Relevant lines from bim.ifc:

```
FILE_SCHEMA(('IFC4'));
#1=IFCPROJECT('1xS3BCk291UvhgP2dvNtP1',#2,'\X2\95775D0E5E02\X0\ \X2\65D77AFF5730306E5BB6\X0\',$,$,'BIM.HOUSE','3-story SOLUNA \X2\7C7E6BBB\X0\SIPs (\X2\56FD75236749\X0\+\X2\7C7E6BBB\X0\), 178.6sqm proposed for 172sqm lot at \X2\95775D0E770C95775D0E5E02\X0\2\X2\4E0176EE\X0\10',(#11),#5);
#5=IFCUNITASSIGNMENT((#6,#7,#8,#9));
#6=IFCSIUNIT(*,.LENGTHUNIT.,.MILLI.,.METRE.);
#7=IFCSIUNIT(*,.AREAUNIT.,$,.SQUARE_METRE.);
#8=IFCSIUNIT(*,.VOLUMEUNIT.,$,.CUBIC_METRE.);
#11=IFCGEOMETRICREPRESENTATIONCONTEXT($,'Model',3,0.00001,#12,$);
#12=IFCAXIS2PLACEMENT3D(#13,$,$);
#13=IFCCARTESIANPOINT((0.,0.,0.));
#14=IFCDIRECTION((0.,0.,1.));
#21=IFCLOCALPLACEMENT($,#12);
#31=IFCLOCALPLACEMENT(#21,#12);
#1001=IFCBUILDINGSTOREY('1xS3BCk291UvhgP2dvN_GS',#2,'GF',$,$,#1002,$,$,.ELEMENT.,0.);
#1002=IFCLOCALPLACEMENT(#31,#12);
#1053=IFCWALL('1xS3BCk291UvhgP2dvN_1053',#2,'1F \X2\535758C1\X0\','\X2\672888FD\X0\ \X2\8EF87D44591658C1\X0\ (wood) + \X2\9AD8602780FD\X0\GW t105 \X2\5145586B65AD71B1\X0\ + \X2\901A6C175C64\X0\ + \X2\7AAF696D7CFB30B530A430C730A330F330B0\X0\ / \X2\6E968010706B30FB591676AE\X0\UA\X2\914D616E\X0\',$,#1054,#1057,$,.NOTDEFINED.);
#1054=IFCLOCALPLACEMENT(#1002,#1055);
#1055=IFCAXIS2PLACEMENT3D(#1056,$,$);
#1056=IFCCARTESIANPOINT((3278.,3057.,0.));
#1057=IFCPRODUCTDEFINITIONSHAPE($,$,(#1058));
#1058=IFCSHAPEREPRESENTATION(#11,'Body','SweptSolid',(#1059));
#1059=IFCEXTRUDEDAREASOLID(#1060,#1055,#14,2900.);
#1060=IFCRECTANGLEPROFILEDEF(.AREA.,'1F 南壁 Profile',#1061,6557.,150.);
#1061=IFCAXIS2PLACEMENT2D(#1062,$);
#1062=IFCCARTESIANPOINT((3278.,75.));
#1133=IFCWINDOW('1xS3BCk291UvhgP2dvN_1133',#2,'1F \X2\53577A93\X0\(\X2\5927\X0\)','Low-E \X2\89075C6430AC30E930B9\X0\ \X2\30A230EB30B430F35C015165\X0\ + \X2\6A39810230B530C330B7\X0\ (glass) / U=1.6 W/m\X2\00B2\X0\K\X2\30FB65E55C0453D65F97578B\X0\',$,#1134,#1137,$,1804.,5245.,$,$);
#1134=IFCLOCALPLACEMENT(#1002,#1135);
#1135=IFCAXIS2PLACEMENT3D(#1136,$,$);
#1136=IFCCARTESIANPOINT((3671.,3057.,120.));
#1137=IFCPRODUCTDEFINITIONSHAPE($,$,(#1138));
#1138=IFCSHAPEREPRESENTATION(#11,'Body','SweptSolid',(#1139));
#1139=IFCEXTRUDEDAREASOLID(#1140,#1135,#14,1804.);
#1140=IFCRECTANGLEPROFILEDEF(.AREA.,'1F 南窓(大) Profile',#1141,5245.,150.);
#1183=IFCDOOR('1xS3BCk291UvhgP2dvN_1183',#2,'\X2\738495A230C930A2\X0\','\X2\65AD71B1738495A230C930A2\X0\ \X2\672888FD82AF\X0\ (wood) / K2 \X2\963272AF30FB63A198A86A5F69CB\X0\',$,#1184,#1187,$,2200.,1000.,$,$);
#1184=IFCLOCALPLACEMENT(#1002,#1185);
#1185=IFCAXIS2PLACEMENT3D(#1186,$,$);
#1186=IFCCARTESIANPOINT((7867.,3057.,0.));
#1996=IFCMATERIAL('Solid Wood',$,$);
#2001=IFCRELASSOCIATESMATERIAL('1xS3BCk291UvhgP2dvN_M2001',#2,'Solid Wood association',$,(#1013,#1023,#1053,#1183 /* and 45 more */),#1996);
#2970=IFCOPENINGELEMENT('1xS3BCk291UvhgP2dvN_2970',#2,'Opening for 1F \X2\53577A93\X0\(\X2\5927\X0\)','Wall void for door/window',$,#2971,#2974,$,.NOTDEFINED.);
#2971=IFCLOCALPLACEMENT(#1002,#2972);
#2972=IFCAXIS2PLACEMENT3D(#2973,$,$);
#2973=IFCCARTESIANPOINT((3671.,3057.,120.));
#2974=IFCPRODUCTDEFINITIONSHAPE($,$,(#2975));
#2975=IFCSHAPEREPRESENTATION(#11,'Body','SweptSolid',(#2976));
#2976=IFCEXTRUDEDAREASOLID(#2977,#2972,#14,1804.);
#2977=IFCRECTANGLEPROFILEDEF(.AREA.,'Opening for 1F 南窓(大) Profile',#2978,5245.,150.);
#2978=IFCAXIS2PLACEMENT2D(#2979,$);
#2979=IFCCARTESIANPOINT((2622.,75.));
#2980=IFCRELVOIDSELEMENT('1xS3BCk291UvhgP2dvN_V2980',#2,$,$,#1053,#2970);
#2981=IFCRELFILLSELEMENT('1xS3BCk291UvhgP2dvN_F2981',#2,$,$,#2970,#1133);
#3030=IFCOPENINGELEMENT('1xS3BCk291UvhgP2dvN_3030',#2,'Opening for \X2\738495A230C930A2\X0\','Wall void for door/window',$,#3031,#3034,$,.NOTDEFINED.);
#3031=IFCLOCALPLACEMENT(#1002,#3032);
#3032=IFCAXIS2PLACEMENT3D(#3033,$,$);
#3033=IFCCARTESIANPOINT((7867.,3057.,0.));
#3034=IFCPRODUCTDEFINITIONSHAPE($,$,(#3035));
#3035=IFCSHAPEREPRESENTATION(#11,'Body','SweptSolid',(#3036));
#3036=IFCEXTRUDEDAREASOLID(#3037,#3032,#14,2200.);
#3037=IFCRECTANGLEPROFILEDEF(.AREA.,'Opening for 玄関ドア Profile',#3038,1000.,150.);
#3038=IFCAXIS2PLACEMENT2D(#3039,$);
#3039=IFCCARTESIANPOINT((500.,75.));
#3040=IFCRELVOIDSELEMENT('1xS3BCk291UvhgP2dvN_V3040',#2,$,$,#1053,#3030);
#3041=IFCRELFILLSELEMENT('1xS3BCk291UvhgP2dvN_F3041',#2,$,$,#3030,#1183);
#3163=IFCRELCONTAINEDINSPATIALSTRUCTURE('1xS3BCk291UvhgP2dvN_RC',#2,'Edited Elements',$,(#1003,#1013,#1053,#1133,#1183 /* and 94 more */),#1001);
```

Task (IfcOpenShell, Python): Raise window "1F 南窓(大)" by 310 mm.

```python
import numpy as np
import ifcopenshell
import ifcopenshell.api.geometry
import ifcopenshell.util.placement
import ifcopenshell.util.unit

model = ifcopenshell.open("bim.ifc")
unit_scale = ifcopenshell.util.unit.calculate_unit_scale(model)

window = model.by_id(1133)
opening = window.FillsVoids[0].RelatingOpeningElement
dz = 0.31 / unit_scale

shift = np.array([0.0, 0.0, dz])
# The window is not placed relative to its opening, so move both.
for product in (opening, window):
    matrix = ifcopenshell.util.placement.get_local_placement(product.ObjectPlacement)
    matrix[:3, 3] += shift
    ifcopenshell.api.geometry.edit_object_placement(model, product=product, matrix=matrix, is_si=False)

print(f"moved by {dz * unit_scale:+.3f} m")

model.write("bim_rev.ifc")
```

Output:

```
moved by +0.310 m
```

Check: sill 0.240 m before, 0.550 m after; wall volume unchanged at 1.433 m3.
